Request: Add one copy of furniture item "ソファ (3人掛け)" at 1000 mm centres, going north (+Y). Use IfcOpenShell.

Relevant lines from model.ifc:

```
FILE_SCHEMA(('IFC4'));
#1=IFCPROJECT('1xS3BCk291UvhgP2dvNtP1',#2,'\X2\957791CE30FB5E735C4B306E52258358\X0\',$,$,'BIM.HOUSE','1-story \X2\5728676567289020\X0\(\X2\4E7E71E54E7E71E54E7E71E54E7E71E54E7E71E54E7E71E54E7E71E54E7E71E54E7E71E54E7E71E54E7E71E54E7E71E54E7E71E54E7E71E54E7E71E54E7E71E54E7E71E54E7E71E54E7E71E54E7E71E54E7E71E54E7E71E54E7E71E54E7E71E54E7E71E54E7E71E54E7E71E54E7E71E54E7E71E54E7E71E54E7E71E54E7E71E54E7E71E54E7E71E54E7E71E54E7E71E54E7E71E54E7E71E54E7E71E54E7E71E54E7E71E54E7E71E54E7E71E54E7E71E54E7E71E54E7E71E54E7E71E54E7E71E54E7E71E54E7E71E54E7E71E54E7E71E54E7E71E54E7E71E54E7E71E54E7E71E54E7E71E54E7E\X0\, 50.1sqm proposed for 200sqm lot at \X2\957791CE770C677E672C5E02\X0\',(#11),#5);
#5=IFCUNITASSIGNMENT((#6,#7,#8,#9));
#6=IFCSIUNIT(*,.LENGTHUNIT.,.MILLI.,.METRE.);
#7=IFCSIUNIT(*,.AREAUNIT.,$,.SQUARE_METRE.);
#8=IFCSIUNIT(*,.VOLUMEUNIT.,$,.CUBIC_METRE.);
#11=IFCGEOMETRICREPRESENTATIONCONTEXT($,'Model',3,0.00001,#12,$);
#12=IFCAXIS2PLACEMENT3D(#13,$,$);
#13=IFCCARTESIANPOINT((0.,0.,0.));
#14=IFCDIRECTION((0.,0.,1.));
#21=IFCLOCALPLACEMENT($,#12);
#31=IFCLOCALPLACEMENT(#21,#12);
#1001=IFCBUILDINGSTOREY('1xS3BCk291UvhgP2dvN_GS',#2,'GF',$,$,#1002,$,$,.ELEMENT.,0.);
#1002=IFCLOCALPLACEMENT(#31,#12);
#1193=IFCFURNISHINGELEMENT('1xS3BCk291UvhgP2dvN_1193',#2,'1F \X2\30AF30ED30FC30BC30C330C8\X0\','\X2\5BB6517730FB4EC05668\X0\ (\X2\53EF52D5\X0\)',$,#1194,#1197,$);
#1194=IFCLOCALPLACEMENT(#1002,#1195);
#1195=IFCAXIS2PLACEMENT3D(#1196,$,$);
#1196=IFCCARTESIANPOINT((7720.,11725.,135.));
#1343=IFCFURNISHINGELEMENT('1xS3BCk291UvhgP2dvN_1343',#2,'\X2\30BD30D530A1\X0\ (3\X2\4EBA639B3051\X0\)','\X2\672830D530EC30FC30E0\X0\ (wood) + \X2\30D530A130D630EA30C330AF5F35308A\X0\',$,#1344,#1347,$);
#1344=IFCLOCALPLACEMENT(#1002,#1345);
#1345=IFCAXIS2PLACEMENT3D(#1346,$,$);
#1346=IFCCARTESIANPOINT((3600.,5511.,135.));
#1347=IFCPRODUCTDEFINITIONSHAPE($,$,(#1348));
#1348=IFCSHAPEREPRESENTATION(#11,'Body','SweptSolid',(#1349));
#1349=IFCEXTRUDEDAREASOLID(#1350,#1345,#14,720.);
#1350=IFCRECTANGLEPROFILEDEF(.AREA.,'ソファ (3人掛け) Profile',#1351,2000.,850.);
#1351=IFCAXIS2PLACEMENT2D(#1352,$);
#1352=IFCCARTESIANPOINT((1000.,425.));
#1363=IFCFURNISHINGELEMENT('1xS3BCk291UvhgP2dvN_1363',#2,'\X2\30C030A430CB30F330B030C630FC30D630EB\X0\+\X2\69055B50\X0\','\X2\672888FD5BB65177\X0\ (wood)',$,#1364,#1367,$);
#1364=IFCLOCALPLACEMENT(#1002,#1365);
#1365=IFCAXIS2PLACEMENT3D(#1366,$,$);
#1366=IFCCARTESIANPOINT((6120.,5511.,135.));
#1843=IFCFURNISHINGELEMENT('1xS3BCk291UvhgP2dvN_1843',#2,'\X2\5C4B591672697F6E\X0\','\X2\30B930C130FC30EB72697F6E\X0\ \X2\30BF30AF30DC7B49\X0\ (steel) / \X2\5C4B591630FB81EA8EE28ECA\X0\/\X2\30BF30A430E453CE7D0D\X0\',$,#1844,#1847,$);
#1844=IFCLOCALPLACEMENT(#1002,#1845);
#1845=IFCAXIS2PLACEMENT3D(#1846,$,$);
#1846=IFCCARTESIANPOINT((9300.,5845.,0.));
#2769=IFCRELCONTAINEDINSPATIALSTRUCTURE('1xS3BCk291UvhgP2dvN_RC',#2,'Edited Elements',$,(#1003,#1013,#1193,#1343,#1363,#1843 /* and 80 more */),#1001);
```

```python
import numpy as np
import ifcopenshell
import ifcopenshell.api.geometry
import ifcopenshell.api.root
import ifcopenshell.util.element
import ifcopenshell.util.placement
import ifcopenshell.util.unit

model = ifcopenshell.open("model.ifc")
unit_scale = ifcopenshell.util.unit.calculate_unit_scale(model)


def reuse_history(source, copy):
    """copy_class also copies each property set's owner history, people and application; keep the originals."""
    for rel in copy.IsDefinedBy:
        if rel.is_a("IfcRelDefinesByProperties") and (history := rel.RelatingPropertyDefinition.OwnerHistory):
            rel.RelatingPropertyDefinition.OwnerHistory = source.OwnerHistory
            ifcopenshell.util.element.remove_deep2(model, history)


source = model.by_guid("1xS3BCk291UvhgP2dvN_1343")
base = ifcopenshell.util.placement.get_local_placement(source.ObjectPlacement)
step = np.array([0.0, 1.0, 0.0]) * 1 / unit_scale

for i in range(1, 2):
    copy = ifcopenshell.api.root.copy_class(model, product=source)
    copy.Representation = ifcopenshell.util.element.copy_deep(
        model, source.Representation, exclude=["IfcGeometricRepresentationContext", "IfcRepresentationMap"]
    )
    reuse_history(source, copy)
    matrix = base.copy()
    matrix[:3, 3] += i * step
    print("added at", matrix[:3, 3].round(3) + 0.0)
    ifcopenshell.api.geometry.edit_object_placement(model, product=copy, matrix=matrix, is_si=False)

model.write("model_v2.ifc")
```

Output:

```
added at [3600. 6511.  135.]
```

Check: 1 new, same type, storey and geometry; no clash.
